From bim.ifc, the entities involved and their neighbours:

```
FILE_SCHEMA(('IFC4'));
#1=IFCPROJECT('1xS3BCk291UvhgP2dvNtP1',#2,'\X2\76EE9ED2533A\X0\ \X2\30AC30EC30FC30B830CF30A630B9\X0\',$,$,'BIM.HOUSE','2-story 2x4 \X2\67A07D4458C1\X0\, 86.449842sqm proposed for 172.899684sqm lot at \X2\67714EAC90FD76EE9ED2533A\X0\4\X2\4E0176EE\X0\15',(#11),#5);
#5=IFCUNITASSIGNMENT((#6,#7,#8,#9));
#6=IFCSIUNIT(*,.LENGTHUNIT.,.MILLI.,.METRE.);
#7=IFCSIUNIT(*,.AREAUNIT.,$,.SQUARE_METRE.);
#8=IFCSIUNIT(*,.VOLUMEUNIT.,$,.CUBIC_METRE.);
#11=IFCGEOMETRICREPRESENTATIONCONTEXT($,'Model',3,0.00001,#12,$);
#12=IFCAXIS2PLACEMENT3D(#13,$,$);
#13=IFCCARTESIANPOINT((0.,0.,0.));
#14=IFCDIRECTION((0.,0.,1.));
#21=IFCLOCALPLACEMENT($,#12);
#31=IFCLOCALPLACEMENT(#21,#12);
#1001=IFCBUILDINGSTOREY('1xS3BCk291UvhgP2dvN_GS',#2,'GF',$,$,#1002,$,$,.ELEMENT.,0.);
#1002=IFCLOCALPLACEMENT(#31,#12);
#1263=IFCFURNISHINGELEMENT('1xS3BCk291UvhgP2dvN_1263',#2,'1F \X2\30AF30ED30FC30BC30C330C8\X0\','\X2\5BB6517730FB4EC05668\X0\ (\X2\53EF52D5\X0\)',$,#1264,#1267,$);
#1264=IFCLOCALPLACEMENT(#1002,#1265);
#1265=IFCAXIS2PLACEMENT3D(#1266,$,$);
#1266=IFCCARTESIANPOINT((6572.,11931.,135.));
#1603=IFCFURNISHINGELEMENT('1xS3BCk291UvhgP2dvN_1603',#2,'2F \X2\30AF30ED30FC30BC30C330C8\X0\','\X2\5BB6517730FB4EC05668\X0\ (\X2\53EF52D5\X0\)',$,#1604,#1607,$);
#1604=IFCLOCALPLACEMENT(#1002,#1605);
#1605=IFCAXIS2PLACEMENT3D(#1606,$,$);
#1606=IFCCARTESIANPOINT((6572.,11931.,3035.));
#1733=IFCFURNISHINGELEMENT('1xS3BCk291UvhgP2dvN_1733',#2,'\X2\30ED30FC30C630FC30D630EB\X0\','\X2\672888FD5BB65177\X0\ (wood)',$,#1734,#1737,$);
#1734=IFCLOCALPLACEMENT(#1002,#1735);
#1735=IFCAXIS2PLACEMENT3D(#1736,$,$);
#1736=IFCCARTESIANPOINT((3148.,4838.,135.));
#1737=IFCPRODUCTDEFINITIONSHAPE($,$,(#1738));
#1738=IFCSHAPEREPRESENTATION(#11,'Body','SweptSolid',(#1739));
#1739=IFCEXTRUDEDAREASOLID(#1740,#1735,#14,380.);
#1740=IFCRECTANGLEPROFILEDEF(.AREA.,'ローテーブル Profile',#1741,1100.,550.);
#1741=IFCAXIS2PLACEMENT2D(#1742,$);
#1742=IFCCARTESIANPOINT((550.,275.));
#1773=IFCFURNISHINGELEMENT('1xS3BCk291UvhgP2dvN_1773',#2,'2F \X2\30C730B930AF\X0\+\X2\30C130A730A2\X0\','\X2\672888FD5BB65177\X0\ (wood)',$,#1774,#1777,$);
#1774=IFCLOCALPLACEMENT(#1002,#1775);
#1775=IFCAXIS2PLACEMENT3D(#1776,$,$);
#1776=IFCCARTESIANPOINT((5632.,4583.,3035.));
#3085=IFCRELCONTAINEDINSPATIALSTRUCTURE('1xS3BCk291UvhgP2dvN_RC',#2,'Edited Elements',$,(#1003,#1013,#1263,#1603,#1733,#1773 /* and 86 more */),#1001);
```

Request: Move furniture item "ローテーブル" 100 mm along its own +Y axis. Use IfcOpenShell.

```python
import ifcopenshell
import ifcopenshell.api.geometry
import ifcopenshell.util.placement
import ifcopenshell.util.unit

model = ifcopenshell.open("bim.ifc")
unit_scale = ifcopenshell.util.unit.calculate_unit_scale(model)

item = model.by_guid("1xS3BCk291UvhgP2dvN_1733")
matrix = ifcopenshell.util.placement.get_local_placement(item.ObjectPlacement)
matrix[:3, 3] += matrix[:3, 1] * 0.1 / unit_scale
ifcopenshell.api.geometry.edit_object_placement(model, product=item, matrix=matrix, is_si=False)

print(ifcopenshell.util.placement.get_local_placement(item.ObjectPlacement).round(3) + 0.0)

model.write("bim_rev.ifc")
```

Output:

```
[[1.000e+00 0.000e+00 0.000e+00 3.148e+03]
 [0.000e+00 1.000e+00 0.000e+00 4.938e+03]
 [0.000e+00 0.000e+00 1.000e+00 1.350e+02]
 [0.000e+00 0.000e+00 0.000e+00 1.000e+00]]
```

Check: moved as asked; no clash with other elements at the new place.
